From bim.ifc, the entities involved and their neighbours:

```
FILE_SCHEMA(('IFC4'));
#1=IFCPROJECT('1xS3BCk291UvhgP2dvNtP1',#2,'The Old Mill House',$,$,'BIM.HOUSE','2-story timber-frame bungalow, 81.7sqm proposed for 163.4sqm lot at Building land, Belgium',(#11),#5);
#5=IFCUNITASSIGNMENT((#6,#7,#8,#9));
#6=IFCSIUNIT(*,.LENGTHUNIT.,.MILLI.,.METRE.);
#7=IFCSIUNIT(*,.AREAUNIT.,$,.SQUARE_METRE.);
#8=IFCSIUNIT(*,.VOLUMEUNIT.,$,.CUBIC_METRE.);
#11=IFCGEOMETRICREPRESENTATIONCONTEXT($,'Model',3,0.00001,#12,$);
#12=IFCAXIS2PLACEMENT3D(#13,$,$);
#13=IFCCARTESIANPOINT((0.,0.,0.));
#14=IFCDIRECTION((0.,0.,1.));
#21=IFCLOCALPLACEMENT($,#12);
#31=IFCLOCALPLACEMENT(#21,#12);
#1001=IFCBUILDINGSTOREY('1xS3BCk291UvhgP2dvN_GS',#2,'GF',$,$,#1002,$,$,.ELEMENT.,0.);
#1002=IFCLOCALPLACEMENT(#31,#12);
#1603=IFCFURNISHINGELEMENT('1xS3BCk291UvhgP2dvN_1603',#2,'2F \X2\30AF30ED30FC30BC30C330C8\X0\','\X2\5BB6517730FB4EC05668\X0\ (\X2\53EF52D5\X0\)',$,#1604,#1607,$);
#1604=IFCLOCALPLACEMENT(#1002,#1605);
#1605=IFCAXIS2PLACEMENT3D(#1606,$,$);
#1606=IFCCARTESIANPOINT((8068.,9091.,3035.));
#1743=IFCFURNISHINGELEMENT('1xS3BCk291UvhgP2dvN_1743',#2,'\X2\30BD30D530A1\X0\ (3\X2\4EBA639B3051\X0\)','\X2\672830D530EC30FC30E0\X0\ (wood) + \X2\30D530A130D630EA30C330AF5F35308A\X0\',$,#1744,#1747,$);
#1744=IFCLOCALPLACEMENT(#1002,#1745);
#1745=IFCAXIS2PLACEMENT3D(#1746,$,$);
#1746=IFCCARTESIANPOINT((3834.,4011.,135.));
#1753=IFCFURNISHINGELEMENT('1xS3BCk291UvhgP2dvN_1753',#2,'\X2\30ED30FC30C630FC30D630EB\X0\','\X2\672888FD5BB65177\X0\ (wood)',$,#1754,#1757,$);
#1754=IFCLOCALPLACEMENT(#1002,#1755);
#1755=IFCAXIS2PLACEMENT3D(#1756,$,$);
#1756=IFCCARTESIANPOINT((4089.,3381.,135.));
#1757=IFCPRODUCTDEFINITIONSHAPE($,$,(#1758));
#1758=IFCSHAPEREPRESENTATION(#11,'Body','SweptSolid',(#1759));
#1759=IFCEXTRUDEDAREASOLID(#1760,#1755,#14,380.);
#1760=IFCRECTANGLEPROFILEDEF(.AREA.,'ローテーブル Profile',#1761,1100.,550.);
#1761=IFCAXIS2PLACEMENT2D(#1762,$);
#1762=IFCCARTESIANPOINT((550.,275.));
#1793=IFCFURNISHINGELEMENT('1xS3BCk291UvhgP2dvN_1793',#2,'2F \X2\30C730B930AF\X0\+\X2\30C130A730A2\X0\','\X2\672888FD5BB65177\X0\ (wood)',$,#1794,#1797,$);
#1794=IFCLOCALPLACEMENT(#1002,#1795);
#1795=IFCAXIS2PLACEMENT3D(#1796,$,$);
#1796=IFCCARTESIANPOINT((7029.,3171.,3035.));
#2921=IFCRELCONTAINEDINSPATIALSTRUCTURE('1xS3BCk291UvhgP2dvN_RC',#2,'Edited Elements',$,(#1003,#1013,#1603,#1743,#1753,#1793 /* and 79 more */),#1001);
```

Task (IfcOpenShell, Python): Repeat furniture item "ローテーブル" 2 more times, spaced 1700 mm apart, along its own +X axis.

```python
import ifcopenshell
import ifcopenshell.api.geometry
import ifcopenshell.api.root
import ifcopenshell.util.element
import ifcopenshell.util.placement
import ifcopenshell.util.unit

model = ifcopenshell.open("bim.ifc")
unit_scale = ifcopenshell.util.unit.calculate_unit_scale(model)


def reuse_history(source, copy):
    """copy_class also copies each property set's owner history, people and application; keep the originals."""
    for rel in copy.IsDefinedBy:
        if rel.is_a("IfcRelDefinesByProperties") and (history := rel.RelatingPropertyDefinition.OwnerHistory):
            rel.RelatingPropertyDefinition.OwnerHistory = source.OwnerHistory
            ifcopenshell.util.element.remove_deep2(model, history)


source = model.by_id(1753)
base = ifcopenshell.util.placement.get_local_placement(source.ObjectPlacement)
step = base[:3, 0] * 1.7 / unit_scale

for i in range(1, 3):
    copy = ifcopenshell.api.root.copy_class(model, product=source)
    copy.Representation = ifcopenshell.util.element.copy_deep(
        model, source.Representation, exclude=["IfcGeometricRepresentationContext", "IfcRepresentationMap"]
    )
    reuse_history(source, copy)
    matrix = base.copy()
    matrix[:3, 3] += i * step
    print("added at", matrix[:3, 3].round(3) + 0.0)
    ifcopenshell.api.geometry.edit_object_placement(model, product=copy, matrix=matrix, is_si=False)

model.write("bim_edited.ifc")
```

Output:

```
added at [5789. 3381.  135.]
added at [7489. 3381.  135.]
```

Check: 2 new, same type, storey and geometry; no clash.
